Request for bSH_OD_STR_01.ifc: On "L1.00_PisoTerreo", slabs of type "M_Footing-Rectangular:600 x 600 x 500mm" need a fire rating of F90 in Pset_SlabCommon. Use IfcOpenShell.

First a look at what the model holds.

```python
import ifcopenshell
import ifcopenshell.util.element

model = ifcopenshell.open("bSH_OD_STR_01.ifc")
print(model.schema)
storey = next(s for s in model.by_type("IfcBuildingStorey") if s.Name == "L1.00_PisoTerreo")
slabs = [e for e in ifcopenshell.util.element.get_decomposition(storey) if e.is_a("IfcSlab")]
seen = {}
for e in slabs:
    element_type = ifcopenshell.util.element.get_type(e)
    key = (element_type.Name if element_type != e and element_type else None, ifcopenshell.util.element.get_pset(e, "Pset_SlabCommon", "FireRating"))
    seen[key] = seen.get(key, 0) + 1
for (name, value), count in sorted(seen.items(), key=str):
    print(count, "x", name, "|", value)
```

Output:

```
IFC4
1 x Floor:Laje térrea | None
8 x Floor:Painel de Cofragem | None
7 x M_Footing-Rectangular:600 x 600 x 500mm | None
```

```python
import ifcopenshell
import ifcopenshell.api.pset
import ifcopenshell.util.element

model = ifcopenshell.open("bSH_OD_STR_01.ifc")

storey = next(s for s in model.by_type("IfcBuildingStorey") if s.Name == "L1.00_PisoTerreo")
slabs = [e for e in ifcopenshell.util.element.get_decomposition(storey) if e.is_a("IfcSlab")]

count = 0
for e in slabs:
    element_type = ifcopenshell.util.element.get_type(e)
    if element_type in (None, e) or element_type.Name != "M_Footing-Rectangular:600 x 600 x 500mm":
        continue
    # add_pset returns the element's existing set when there is one.
    pset = ifcopenshell.api.pset.add_pset(model, product=e, name="Pset_SlabCommon")
    ifcopenshell.api.pset.edit_pset(model, pset=pset, properties={"FireRating": "F90"})
    count += 1

print(count, "slabs updated")

model.write("bSH_OD_STR_01_updated.ifc")
```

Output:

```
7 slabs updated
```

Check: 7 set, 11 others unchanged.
